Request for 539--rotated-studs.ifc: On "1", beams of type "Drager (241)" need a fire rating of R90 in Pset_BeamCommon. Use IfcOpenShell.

First a look at what the model holds.

```python
import ifcopenshell
import ifcopenshell.util.element

model = ifcopenshell.open("539--rotated-studs.ifc")
print(model.schema)
storey = next(s for s in model.by_type("IfcBuildingStorey") if s.Name == "1")
beams = [e for e in ifcopenshell.util.element.get_decomposition(storey) if e.is_a("IfcBeam")]
seen = {}
for e in beams:
    element_type = ifcopenshell.util.element.get_type(e)
    key = (element_type.Name if element_type != e and element_type else None, ifcopenshell.util.element.get_pset(e, "Pset_BeamCommon", "FireRating"))
    seen[key] = seen.get(key, 0) + 1
for (name, value), count in sorted(seen.items(), key=str):
    print(count, "x", name, "|", value)
```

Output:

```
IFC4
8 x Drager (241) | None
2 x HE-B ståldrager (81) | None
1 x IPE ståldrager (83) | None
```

```python
import ifcopenshell
import ifcopenshell.api.pset
import ifcopenshell.util.element

model = ifcopenshell.open("539--rotated-studs.ifc")

storey = next(s for s in model.by_type("IfcBuildingStorey") if s.Name == "1")
beams = [e for e in ifcopenshell.util.element.get_decomposition(storey) if e.is_a("IfcBeam")]

count = 0
for e in beams:
    element_type = ifcopenshell.util.element.get_type(e)
    if element_type in (None, e) or element_type.Name != "Drager (241)":
        continue
    # add_pset returns the element's existing set when there is one.
    pset = ifcopenshell.api.pset.add_pset(model, product=e, name="Pset_BeamCommon")
    ifcopenshell.api.pset.edit_pset(model, pset=pset, properties={"FireRating": "R90"})
    count += 1

print(count, "beams updated")

model.write("539--rotated-studs-out.ifc")
```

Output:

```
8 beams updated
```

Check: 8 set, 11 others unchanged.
